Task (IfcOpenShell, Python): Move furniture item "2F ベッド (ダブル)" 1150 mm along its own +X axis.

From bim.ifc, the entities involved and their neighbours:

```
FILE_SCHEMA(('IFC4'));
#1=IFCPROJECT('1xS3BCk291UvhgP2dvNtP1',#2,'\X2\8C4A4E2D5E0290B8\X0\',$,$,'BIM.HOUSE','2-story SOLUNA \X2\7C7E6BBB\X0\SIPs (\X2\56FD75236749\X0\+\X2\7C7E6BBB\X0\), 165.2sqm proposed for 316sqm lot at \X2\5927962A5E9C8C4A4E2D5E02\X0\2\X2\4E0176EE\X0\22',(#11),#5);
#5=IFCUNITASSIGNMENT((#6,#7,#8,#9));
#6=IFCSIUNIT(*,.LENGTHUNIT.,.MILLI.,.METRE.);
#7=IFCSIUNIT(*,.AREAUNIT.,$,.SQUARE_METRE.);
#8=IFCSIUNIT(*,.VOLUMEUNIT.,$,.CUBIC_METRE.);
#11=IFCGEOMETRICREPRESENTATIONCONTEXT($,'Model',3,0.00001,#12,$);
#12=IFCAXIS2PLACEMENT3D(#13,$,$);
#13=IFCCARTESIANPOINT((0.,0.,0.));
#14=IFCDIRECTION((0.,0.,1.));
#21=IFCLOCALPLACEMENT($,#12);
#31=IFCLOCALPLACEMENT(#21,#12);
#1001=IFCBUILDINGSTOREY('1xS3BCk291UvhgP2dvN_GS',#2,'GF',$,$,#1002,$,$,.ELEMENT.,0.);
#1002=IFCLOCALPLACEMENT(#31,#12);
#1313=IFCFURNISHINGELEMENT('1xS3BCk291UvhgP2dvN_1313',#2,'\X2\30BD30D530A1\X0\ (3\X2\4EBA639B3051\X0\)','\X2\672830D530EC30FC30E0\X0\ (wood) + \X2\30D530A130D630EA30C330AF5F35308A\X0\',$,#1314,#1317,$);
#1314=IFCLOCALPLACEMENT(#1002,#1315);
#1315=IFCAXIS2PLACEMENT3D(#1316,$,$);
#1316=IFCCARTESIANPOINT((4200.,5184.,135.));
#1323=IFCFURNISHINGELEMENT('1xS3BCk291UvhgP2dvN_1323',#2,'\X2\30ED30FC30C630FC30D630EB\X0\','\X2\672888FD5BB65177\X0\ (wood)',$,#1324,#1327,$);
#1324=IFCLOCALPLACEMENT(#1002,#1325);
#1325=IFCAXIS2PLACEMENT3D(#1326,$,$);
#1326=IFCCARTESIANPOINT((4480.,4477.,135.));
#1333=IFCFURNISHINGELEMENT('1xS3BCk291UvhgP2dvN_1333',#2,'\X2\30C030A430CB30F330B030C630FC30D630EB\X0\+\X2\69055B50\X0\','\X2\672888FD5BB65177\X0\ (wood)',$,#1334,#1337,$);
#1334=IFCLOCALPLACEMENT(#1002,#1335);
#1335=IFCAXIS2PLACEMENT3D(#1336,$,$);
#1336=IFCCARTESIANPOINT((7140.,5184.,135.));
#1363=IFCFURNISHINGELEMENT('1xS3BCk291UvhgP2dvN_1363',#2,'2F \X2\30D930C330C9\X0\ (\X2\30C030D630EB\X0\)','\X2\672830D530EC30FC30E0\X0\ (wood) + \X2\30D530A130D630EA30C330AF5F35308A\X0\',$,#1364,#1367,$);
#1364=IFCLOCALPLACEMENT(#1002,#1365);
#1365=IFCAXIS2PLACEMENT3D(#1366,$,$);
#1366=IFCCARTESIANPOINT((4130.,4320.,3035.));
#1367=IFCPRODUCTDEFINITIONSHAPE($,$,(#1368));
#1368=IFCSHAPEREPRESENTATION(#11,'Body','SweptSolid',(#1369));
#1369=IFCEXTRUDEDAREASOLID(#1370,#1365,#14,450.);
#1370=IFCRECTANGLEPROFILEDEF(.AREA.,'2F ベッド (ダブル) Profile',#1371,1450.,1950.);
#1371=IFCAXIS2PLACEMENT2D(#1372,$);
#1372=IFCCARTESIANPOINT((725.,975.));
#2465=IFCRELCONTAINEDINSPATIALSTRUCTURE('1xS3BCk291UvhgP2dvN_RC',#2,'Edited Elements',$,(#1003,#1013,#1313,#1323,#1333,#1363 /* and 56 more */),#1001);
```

```python
import ifcopenshell
import ifcopenshell.api.geometry
import ifcopenshell.util.placement
import ifcopenshell.util.unit

model = ifcopenshell.open("bim.ifc")
unit_scale = ifcopenshell.util.unit.calculate_unit_scale(model)

item = model.by_guid("1xS3BCk291UvhgP2dvN_1363")
matrix = ifcopenshell.util.placement.get_local_placement(item.ObjectPlacement)
matrix[:3, 3] += matrix[:3, 0] * 1.15 / unit_scale
ifcopenshell.api.geometry.edit_object_placement(model, product=item, matrix=matrix, is_si=False)

print(ifcopenshell.util.placement.get_local_placement(item.ObjectPlacement).round(3) + 0.0)

model.write("bim_v2.ifc")
```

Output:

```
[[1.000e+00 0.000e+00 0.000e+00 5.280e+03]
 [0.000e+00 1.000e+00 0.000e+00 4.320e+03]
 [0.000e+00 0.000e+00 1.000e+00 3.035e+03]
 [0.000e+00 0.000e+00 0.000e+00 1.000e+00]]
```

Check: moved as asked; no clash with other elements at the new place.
